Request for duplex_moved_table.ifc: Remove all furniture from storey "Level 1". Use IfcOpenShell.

First a look at what the model holds.

```python
import ifcopenshell
import ifcopenshell.util.element

model = ifcopenshell.open("duplex_moved_table.ifc")
print(model.schema)
storey = next(s for s in model.by_type("IfcBuildingStorey") if s.Name == "Level 1")
furniture = [e for e in ifcopenshell.util.element.get_decomposition(storey) if e.is_a("IfcFurnishingElement")]
seen = {}
for e in furniture:
    element_type = ifcopenshell.util.element.get_type(e)
    name = element_type.Name if element_type not in (None, e) else None
    seen[name] = seen.get(name, 0) + 1
for name, count in sorted(seen.items(), key=str):
    print(count, "x", name)
```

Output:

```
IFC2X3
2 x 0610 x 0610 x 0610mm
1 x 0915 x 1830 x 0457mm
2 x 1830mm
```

```python
import ifcopenshell
import ifcopenshell.api.root
import ifcopenshell.util.element

model = ifcopenshell.open("duplex_moved_table.ifc")

storey = next(s for s in model.by_type("IfcBuildingStorey") if s.Name == "Level 1")
furniture = [e for e in ifcopenshell.util.element.get_decomposition(storey) if e.is_a("IfcFurnishingElement")]

for e in furniture:
    ifcopenshell.api.root.remove_product(model, product=e)
print(len(furniture), "removed")

model.write("duplex_moved_table_v2.ifc")
```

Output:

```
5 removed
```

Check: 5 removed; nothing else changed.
